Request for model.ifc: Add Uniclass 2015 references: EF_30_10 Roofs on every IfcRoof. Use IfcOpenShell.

First a look at what the model holds.

```python
import ifcopenshell

model = ifcopenshell.open("model.ifc")
print(model.schema)
print("classifications:", [c.Name for c in model.by_type("IfcClassification")])
for ifc_class in ("IfcDoor", "IfcRoof", "IfcStair", "IfcWall", "IfcWindow"):
    print(ifc_class, len(model.by_type(ifc_class)))
```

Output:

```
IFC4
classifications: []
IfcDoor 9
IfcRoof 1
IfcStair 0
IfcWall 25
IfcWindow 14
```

```python
import ifcopenshell
import ifcopenshell.api.classification

model = ifcopenshell.open("model.ifc")

system = ifcopenshell.api.classification.add_classification(model, classification="Uniclass 2015")

codes = {
    "IfcRoof": ("EF_30_10", "Roofs"),
}
for ifc_class, (code, name) in codes.items():
    products = model.by_type(ifc_class)
    ifcopenshell.api.classification.add_reference(
        model, products=products, classification=system, identification=code, name=name
    )
    print(code, len(products))

model.write("model_updated.ifc")
```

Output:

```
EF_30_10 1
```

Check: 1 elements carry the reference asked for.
